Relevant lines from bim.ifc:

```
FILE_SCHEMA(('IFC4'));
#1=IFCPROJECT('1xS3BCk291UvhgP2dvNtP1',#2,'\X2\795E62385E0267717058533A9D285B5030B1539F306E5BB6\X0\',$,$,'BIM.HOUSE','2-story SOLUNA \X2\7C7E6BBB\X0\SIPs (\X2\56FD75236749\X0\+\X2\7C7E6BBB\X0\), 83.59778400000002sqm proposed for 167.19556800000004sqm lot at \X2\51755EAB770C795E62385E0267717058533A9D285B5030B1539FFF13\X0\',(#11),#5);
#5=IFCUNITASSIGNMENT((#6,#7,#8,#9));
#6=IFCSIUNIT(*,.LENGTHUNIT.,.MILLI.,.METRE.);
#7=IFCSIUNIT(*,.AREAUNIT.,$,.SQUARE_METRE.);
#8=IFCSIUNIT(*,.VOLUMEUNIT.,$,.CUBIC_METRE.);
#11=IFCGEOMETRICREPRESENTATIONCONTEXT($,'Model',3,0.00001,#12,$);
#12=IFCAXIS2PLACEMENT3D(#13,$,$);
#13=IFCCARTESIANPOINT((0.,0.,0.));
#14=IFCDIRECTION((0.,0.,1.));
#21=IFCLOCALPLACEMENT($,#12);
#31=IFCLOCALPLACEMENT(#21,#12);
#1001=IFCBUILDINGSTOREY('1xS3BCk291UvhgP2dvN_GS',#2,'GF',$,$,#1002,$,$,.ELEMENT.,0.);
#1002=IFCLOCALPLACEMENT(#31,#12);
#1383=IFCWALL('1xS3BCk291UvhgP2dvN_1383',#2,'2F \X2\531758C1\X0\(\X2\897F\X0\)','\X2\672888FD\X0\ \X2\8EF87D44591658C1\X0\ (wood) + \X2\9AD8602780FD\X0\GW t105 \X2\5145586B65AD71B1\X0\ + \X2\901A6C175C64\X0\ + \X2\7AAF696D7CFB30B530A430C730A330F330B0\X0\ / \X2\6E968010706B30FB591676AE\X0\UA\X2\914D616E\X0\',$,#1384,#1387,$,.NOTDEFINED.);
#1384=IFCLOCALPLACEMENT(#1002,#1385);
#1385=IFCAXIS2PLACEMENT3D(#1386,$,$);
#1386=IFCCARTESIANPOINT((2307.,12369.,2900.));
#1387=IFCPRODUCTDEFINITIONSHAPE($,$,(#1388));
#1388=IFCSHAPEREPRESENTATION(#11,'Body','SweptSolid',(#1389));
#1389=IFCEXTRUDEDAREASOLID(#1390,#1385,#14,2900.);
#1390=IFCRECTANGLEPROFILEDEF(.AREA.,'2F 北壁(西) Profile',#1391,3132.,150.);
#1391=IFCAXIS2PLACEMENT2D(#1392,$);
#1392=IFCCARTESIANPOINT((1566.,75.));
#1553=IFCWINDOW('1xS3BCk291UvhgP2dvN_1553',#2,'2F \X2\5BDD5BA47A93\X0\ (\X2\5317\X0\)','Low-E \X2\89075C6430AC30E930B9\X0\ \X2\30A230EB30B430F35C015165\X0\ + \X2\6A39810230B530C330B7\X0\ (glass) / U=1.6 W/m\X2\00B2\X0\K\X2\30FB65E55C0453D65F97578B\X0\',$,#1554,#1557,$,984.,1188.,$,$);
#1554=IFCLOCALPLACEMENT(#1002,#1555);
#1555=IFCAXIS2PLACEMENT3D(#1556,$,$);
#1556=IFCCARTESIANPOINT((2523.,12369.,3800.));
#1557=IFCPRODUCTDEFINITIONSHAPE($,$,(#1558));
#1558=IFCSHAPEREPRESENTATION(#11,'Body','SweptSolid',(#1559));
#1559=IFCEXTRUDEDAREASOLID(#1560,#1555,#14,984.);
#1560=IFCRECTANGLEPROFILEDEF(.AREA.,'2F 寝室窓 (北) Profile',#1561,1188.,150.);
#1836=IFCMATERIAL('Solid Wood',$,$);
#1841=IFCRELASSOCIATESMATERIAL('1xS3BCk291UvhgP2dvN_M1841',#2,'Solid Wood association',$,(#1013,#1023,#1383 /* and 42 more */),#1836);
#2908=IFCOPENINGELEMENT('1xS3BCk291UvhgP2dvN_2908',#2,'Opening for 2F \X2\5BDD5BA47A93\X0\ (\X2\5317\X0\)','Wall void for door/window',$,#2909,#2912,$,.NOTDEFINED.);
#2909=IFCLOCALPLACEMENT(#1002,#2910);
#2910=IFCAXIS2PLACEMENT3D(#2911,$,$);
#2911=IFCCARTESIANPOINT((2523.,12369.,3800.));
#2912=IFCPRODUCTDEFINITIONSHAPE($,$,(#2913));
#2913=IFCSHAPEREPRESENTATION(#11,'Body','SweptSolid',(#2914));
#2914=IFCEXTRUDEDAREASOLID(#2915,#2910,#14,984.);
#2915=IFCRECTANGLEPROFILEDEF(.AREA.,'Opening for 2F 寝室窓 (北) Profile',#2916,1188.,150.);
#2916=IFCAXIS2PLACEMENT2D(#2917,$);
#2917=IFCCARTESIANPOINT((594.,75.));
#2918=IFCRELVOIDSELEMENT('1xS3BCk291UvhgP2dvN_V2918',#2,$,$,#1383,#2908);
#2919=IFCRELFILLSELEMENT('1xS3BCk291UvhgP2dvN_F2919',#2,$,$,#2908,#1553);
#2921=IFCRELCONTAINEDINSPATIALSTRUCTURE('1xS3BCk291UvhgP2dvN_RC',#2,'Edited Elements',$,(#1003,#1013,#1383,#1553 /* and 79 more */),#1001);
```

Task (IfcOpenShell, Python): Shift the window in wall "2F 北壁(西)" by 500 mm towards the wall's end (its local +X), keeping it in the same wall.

```python
import ifcopenshell
import ifcopenshell.api.geometry
import ifcopenshell.util.placement

model = ifcopenshell.open("bim.ifc")

window = model.by_guid("1xS3BCk291UvhgP2dvN_1553")
opening = window.FillsVoids[0].RelatingOpeningElement
wall = opening.VoidsElements[0].RelatingBuildingElement

wall_matrix = ifcopenshell.util.placement.get_local_placement(wall.ObjectPlacement)
shift = wall_matrix[:3, 0] * 500.0
before = ifcopenshell.util.placement.get_local_placement(window.ObjectPlacement)[:3, 3].copy()

# The window is not placed relative to its opening, so move both.
for product in (opening, window):
    matrix = ifcopenshell.util.placement.get_local_placement(product.ObjectPlacement)
    matrix[:3, 3] += shift
    ifcopenshell.api.geometry.edit_object_placement(model, product=product, matrix=matrix, is_si=False)

after = ifcopenshell.util.placement.get_local_placement(window.ObjectPlacement)[:3, 3]
print("window moved by", (after - before).round(3) + 0.0)

model.write("bim-out.ifc")
```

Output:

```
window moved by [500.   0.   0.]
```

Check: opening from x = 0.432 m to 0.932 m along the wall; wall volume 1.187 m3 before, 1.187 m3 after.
